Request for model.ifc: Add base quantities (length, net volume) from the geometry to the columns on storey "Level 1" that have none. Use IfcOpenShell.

First a look at what the model holds.

```python
import ifcopenshell
import ifcopenshell.util.element
import ifcopenshell.util.unit

model = ifcopenshell.open("model.ifc")
print(model.schema)
for unit_type in ("LENGTHUNIT", "AREAUNIT", "VOLUMEUNIT"):
    print(unit_type, ifcopenshell.util.unit.calculate_unit_scale(model, unit_type))
storey = next(s for s in model.by_type("IfcBuildingStorey") if s.Name == "Level 1")
columns = [e for e in ifcopenshell.util.element.get_decomposition(storey) if e.is_a("IfcColumn")]
for e in sorted(columns, key=lambda e: e.id()):
    print(e.id(), e.is_a(), e.Name, list(ifcopenshell.util.element.get_psets(e, qtos_only=True)), sep=" | ")
```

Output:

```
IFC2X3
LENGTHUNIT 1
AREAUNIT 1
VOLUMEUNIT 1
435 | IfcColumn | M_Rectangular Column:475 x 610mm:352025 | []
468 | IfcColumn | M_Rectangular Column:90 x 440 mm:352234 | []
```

```python
import ifcopenshell
import ifcopenshell.api.pset
import ifcopenshell.geom
import ifcopenshell.util.element
import ifcopenshell.util.shape
import ifcopenshell.util.unit

model = ifcopenshell.open("model.ifc")
unit_scale = ifcopenshell.util.unit.calculate_unit_scale(model)
volume_scale = ifcopenshell.util.unit.calculate_unit_scale(model, "VOLUMEUNIT")
settings = ifcopenshell.geom.settings()

storey = next(s for s in model.by_type("IfcBuildingStorey") if s.Name == "Level 1")
columns = [e for e in ifcopenshell.util.element.get_decomposition(storey) if e.is_a("IfcColumn")]

for e in sorted(columns, key=lambda e: e.id()):
    if ifcopenshell.util.element.get_psets(e, qtos_only=True, should_inherit=False):
        continue
    # Geometry comes back in metres, in the element's own axes.
    shape = ifcopenshell.geom.create_shape(settings, e)
    values = {
        "Length": ifcopenshell.util.shape.get_z(shape.geometry) / unit_scale,
        "NetVolume": ifcopenshell.util.shape.get_volume(shape.geometry) / volume_scale,
    }
    qto = ifcopenshell.api.pset.add_qto(model, product=e, name="BaseQuantities")
    ifcopenshell.api.pset.edit_qto(model, qto=qto, properties=values)
    print(e.id(), {k: round(v, 3) for k, v in values.items()})

model.write("model_updated.ifc")
```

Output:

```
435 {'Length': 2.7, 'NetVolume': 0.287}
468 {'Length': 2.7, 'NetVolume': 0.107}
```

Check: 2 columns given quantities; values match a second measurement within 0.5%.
